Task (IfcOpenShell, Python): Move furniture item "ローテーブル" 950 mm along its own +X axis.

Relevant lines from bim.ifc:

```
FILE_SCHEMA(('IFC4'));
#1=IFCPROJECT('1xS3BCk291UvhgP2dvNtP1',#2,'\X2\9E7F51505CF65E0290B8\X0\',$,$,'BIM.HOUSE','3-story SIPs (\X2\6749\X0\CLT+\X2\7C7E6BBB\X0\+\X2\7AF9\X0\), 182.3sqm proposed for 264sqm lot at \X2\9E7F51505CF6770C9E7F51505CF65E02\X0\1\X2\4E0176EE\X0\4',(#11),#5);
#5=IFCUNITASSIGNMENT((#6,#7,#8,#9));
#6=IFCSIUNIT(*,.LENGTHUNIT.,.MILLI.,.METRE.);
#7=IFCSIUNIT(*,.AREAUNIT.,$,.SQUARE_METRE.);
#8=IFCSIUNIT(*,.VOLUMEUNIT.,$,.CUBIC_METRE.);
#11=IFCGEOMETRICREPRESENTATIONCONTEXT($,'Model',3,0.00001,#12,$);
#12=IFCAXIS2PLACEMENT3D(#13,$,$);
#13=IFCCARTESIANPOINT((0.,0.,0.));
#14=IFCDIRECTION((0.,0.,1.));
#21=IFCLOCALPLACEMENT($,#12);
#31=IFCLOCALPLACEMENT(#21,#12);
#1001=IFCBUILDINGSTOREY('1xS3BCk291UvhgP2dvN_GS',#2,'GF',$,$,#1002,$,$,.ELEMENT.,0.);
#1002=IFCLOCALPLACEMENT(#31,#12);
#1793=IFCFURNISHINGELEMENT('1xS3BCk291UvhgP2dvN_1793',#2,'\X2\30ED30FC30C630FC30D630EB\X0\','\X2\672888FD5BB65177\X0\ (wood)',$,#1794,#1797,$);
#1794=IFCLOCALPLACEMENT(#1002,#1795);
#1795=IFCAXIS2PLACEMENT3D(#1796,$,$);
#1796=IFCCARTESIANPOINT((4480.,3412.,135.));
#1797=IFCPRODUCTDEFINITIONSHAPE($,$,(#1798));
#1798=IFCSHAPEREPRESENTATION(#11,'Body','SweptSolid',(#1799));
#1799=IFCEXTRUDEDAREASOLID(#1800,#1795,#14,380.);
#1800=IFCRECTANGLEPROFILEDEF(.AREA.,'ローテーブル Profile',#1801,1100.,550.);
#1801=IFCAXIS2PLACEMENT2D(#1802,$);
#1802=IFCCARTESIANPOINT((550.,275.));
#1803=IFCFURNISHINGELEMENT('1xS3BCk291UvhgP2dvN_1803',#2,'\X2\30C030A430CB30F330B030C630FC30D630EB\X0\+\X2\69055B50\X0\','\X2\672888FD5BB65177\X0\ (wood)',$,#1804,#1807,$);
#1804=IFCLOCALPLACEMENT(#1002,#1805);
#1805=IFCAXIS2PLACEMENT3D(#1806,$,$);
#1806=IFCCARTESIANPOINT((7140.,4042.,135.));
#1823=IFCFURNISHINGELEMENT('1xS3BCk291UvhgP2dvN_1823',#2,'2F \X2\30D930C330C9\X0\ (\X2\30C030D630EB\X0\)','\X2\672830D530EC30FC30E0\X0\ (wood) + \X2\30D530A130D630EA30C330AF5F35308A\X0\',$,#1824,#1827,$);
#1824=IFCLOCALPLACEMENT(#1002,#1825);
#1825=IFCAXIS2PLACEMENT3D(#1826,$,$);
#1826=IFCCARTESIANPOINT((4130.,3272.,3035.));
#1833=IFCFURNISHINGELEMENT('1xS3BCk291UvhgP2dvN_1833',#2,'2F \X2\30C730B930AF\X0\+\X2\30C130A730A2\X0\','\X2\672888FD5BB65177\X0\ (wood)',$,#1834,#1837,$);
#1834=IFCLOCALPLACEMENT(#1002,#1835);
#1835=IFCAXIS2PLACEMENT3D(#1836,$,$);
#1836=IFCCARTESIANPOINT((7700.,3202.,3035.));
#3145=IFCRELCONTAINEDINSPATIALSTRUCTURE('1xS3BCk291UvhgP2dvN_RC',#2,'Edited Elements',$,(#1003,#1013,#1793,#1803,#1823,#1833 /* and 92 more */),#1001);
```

```python
import ifcopenshell
import ifcopenshell.api.geometry
import ifcopenshell.util.placement

model = ifcopenshell.open("bim.ifc")

item = model.by_guid("1xS3BCk291UvhgP2dvN_1793")
matrix = ifcopenshell.util.placement.get_local_placement(item.ObjectPlacement)
matrix[:3, 3] += matrix[:3, 0] * 950.0
ifcopenshell.api.geometry.edit_object_placement(model, product=item, matrix=matrix, is_si=False)

print(ifcopenshell.util.placement.get_local_placement(item.ObjectPlacement).round(3) + 0.0)

model.write("bim_v2.ifc")
```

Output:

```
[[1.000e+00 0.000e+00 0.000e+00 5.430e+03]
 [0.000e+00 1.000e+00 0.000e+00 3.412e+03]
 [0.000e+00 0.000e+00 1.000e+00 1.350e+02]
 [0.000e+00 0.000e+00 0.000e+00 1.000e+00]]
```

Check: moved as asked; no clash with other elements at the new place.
